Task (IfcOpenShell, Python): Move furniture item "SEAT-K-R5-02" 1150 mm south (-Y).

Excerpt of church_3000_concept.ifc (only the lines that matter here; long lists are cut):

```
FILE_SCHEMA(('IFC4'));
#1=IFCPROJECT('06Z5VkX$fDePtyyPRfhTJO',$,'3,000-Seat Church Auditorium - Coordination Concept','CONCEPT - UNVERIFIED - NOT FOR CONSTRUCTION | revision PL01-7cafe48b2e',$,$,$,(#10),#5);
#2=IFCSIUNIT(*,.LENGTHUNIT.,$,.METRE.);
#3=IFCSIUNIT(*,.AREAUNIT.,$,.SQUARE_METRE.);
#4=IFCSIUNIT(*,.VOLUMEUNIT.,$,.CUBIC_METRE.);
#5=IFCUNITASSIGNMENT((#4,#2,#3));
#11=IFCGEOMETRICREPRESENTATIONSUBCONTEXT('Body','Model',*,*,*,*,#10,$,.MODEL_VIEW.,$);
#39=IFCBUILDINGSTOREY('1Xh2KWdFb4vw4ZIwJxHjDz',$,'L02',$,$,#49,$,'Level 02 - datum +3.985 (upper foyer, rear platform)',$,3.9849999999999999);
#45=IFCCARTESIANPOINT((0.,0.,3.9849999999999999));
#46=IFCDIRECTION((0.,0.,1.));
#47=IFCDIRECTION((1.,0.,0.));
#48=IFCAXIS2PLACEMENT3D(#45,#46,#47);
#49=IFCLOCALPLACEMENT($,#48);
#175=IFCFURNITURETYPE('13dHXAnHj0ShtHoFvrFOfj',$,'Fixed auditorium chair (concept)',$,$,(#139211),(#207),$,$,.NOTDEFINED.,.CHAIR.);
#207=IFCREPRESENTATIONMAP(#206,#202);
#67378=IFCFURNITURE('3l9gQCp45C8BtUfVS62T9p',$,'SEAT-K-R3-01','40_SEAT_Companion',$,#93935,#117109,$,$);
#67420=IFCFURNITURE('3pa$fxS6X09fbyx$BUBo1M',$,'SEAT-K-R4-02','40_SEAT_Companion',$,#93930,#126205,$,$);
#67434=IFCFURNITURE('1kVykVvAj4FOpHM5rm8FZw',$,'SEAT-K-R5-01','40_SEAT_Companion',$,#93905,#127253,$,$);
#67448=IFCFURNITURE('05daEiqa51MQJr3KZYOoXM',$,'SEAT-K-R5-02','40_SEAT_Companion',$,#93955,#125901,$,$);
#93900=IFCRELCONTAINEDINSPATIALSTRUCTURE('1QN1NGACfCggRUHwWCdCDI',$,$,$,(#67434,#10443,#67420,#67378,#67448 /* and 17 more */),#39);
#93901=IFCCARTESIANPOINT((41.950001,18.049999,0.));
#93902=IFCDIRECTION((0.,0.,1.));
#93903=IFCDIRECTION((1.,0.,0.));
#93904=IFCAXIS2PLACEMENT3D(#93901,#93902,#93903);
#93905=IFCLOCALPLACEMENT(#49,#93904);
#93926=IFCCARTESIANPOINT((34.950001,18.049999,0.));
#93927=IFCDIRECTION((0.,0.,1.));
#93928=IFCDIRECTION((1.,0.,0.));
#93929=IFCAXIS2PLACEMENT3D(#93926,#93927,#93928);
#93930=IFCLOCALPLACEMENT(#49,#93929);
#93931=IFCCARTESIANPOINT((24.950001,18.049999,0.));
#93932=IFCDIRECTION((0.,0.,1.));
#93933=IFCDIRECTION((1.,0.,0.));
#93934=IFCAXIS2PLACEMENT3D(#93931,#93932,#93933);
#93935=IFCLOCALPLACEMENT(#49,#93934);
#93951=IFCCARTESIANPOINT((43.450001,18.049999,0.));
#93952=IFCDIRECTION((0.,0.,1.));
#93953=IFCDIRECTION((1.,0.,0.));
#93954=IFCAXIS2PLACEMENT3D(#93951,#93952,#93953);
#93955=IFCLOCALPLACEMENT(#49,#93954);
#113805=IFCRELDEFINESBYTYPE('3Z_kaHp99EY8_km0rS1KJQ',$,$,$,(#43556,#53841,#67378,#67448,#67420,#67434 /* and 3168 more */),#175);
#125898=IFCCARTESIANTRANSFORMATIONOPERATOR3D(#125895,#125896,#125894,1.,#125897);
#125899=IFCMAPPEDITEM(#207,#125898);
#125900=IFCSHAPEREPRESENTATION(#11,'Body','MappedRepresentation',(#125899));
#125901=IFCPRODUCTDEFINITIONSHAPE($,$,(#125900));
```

```python
import ifcopenshell
import ifcopenshell.api.geometry
import ifcopenshell.util.placement
import ifcopenshell.util.unit

model = ifcopenshell.open("church_3000_concept.ifc")
unit_scale = ifcopenshell.util.unit.calculate_unit_scale(model)

item = model.by_guid("05daEiqa51MQJr3KZYOoXM")
matrix = ifcopenshell.util.placement.get_local_placement(item.ObjectPlacement)
matrix[1, 3] -= 1.15 / unit_scale
ifcopenshell.api.geometry.edit_object_placement(model, product=item, matrix=matrix, is_si=False)

print(ifcopenshell.util.placement.get_local_placement(item.ObjectPlacement).round(3) + 0.0)

model.write("church_3000_concept_v2.ifc")
```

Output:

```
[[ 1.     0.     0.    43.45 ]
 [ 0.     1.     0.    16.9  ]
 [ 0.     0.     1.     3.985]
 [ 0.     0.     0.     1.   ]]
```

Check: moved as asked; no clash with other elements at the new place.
